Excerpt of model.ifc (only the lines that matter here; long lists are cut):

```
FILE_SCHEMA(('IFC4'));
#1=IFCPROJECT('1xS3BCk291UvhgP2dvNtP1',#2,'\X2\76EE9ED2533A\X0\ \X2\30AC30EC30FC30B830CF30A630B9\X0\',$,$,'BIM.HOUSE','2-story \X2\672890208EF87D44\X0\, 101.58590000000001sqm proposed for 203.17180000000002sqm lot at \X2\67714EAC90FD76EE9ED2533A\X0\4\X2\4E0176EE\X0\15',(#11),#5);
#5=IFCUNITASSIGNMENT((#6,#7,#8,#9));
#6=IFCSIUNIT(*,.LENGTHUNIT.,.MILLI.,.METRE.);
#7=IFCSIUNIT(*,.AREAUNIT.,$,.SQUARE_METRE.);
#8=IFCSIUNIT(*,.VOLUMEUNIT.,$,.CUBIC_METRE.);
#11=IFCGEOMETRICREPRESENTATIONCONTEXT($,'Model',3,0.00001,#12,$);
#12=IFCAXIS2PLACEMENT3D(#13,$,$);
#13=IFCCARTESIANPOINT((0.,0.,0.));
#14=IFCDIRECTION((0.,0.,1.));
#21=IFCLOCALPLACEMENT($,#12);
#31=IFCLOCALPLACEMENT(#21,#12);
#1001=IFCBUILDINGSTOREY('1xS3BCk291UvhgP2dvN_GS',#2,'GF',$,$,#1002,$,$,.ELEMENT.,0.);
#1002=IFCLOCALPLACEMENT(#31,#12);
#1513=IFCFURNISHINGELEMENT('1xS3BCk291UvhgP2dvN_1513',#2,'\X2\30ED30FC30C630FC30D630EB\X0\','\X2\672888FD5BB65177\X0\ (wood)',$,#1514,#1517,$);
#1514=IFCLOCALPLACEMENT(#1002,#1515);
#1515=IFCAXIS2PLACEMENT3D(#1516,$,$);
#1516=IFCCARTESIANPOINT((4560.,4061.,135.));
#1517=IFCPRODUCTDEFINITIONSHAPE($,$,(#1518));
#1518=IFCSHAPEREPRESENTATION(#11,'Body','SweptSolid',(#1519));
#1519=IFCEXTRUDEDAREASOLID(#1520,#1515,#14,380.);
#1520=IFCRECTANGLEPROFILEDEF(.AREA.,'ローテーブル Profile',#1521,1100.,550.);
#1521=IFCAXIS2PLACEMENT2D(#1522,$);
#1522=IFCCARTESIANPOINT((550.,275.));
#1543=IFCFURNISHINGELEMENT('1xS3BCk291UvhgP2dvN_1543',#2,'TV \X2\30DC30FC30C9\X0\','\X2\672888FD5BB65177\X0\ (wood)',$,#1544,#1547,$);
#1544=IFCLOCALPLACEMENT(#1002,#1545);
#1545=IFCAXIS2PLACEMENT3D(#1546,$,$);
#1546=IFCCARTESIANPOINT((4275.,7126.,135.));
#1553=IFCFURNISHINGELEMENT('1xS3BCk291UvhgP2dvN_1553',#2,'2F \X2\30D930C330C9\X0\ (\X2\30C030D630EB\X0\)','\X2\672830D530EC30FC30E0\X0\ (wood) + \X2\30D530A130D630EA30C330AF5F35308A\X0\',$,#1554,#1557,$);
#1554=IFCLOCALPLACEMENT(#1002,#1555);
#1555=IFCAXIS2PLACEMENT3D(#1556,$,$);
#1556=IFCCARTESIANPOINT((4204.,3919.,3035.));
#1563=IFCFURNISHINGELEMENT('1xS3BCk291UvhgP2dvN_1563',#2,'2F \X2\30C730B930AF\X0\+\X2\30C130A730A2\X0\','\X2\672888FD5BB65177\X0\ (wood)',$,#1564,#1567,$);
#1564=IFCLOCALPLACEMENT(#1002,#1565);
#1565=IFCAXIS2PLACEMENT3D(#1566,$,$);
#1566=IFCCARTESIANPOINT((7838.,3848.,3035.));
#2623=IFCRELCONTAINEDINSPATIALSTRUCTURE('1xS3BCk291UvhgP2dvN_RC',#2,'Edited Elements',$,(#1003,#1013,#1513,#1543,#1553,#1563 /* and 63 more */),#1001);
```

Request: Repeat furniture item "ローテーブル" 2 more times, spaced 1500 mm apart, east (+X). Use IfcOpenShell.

```python
import numpy as np
import ifcopenshell
import ifcopenshell.api.geometry
import ifcopenshell.api.root
import ifcopenshell.util.element
import ifcopenshell.util.placement
import ifcopenshell.util.unit

model = ifcopenshell.open("model.ifc")
unit_scale = ifcopenshell.util.unit.calculate_unit_scale(model)


def reuse_history(source, copy):
    """copy_class also copies each property set's owner history, people and application; keep the originals."""
    for rel in copy.IsDefinedBy:
        if rel.is_a("IfcRelDefinesByProperties") and (history := rel.RelatingPropertyDefinition.OwnerHistory):
            rel.RelatingPropertyDefinition.OwnerHistory = source.OwnerHistory
            ifcopenshell.util.element.remove_deep2(model, history)


source = model.by_id(1513)
base = ifcopenshell.util.placement.get_local_placement(source.ObjectPlacement)
step = np.array([1.0, 0.0, 0.0]) * 1.5 / unit_scale

for i in range(1, 3):
    copy = ifcopenshell.api.root.copy_class(model, product=source)
    copy.Representation = ifcopenshell.util.element.copy_deep(
        model, source.Representation, exclude=["IfcGeometricRepresentationContext", "IfcRepresentationMap"]
    )
    reuse_history(source, copy)
    matrix = base.copy()
    matrix[:3, 3] += i * step
    print("added at", matrix[:3, 3].round(3) + 0.0)
    ifcopenshell.api.geometry.edit_object_placement(model, product=copy, matrix=matrix, is_si=False)

model.write("model_v2.ifc")
```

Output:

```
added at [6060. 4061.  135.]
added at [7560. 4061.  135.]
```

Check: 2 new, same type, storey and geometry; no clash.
